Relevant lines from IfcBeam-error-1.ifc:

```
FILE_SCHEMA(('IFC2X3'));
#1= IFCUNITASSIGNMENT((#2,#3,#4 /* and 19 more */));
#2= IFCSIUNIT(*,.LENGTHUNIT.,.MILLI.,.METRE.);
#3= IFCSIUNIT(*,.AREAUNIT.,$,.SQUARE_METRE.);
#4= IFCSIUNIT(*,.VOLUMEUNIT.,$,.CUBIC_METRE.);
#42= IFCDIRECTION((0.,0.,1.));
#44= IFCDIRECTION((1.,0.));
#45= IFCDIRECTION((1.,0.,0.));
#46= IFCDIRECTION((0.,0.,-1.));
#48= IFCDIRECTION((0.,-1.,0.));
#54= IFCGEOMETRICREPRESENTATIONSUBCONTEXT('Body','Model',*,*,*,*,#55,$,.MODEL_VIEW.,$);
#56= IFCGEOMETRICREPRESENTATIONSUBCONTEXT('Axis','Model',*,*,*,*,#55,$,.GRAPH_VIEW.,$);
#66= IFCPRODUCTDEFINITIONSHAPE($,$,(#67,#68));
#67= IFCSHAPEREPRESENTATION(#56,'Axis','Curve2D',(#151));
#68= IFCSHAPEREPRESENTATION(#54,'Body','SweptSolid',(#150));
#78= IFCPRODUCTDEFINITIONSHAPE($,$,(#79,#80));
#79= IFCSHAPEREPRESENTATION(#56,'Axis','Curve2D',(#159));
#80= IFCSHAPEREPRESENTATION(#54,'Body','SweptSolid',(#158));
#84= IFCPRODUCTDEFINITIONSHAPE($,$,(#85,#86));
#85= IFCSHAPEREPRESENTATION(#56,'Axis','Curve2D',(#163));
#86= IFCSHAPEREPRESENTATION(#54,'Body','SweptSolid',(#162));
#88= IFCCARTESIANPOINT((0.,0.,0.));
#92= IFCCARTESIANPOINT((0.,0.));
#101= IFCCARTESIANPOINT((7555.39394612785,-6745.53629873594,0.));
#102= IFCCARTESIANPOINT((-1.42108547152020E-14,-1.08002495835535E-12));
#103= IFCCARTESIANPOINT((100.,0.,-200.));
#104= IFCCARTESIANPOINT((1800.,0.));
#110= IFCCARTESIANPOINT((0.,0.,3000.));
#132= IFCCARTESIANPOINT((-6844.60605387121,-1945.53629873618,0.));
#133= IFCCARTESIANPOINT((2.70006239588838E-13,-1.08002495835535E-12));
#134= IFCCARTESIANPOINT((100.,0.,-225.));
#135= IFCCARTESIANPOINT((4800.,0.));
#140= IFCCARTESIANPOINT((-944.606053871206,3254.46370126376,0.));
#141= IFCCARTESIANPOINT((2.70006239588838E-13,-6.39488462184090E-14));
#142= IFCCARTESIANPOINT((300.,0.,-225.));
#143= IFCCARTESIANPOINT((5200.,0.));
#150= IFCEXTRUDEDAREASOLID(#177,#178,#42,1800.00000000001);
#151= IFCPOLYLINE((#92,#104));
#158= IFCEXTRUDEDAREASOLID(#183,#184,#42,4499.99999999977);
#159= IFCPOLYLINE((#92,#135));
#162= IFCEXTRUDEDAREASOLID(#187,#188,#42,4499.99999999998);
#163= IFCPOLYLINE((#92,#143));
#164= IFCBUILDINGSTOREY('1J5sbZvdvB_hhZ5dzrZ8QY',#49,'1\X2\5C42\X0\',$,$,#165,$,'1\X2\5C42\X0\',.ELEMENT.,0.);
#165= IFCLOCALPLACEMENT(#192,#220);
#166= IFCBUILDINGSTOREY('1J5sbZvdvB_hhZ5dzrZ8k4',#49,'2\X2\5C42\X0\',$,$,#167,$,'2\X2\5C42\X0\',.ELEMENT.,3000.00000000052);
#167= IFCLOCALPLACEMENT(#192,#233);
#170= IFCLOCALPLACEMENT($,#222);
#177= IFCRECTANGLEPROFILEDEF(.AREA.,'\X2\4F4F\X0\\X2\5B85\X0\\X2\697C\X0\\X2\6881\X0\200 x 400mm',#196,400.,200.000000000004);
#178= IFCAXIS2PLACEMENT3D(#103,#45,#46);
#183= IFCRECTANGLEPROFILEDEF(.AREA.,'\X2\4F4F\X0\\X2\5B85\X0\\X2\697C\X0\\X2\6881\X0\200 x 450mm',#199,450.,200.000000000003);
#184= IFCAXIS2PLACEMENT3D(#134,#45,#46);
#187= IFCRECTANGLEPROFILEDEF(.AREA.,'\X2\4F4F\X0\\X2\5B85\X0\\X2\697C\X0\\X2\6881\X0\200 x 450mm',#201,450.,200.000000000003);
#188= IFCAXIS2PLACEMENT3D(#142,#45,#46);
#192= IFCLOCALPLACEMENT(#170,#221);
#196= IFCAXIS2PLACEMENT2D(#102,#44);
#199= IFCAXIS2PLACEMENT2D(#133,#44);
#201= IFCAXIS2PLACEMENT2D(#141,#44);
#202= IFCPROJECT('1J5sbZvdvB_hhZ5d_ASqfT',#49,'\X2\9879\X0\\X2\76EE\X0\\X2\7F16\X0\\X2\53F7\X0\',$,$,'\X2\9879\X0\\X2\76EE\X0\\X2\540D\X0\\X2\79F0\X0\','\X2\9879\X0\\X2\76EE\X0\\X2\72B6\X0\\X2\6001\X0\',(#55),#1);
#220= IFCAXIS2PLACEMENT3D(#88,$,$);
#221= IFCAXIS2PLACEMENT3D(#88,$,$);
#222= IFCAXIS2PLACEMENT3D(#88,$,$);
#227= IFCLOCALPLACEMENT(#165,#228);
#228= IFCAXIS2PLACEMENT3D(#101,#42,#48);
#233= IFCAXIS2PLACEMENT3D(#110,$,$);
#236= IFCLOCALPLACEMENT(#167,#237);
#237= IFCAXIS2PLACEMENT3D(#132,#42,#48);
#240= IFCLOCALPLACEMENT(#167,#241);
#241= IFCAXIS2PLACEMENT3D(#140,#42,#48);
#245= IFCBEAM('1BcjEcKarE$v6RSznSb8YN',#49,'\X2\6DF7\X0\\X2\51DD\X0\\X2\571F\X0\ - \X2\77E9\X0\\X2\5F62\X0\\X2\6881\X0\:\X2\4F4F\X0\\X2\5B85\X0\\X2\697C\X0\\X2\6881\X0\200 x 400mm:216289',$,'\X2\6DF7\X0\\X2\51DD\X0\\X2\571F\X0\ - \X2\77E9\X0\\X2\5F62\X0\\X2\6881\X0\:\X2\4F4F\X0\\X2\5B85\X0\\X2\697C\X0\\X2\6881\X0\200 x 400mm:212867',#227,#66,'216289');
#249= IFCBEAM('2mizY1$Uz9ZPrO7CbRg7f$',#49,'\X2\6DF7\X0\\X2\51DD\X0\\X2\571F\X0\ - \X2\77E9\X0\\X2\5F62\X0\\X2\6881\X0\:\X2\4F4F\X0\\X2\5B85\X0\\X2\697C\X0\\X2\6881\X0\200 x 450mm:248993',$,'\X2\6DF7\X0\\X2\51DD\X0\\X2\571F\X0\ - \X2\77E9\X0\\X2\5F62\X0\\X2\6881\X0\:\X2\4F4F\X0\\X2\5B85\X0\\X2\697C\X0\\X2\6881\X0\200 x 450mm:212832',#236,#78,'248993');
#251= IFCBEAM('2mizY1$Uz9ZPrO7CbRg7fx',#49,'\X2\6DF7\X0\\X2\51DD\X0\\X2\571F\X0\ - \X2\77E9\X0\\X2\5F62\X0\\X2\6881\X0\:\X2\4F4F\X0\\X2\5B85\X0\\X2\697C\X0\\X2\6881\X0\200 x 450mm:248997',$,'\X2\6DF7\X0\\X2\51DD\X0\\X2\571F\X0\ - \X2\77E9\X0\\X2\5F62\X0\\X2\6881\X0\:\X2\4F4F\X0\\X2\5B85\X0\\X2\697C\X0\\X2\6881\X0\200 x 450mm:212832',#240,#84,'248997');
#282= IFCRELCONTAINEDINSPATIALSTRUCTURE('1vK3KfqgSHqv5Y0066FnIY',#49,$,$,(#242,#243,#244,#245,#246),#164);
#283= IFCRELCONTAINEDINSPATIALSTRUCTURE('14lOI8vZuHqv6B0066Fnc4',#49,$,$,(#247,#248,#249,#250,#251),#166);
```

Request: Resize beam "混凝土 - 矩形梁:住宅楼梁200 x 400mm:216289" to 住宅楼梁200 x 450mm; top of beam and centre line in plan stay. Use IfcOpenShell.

```python
import ifcopenshell
import ifcopenshell.util.element
import ifcopenshell.util.representation

model = ifcopenshell.open("IfcBeam-error-1.ifc")

member = model.by_guid("1BcjEcKarE$v6RSznSb8YN")
source = next(p for p in model.by_type("IfcRectangleProfileDef") if p.ProfileName == "住宅楼梁200 x 450mm")

body = ifcopenshell.util.representation.get_representation(member, "Model", "Body")
solid = body.Items[0]
old_profile = solid.SweptArea

# Copy the section's sizes but keep this member's own profile position.
profile = ifcopenshell.util.element.copy(model, source)
# Profiles are centred, so shift by half the change in depth to hold the top.
shift = (old_profile.XDim - profile.XDim) / 2
x, y = old_profile.Position.Location.Coordinates
up = (-1.0, 0.0)  # upwards, in the solid's own plane
location = model.createIfcCartesianPoint((x + up[0] * shift, y + up[1] * shift))
profile.Position = model.createIfcAxis2Placement2D(location, old_profile.Position.RefDirection)
solid.SweptArea = profile
if not model.get_total_inverses(old_profile):
    ifcopenshell.util.element.remove_deep2(model, old_profile)
member.Name = member.Name.replace("住宅楼梁200 x 400mm", "住宅楼梁200 x 450mm")
member.ObjectType = member.ObjectType.replace("住宅楼梁200 x 400mm", "住宅楼梁200 x 450mm")

print(solid.SweptArea)

model.write("IfcBeam-error-1_edited.ifc")
```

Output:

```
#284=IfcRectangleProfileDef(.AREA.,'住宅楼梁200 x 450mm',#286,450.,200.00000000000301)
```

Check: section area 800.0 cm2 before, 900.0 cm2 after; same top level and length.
